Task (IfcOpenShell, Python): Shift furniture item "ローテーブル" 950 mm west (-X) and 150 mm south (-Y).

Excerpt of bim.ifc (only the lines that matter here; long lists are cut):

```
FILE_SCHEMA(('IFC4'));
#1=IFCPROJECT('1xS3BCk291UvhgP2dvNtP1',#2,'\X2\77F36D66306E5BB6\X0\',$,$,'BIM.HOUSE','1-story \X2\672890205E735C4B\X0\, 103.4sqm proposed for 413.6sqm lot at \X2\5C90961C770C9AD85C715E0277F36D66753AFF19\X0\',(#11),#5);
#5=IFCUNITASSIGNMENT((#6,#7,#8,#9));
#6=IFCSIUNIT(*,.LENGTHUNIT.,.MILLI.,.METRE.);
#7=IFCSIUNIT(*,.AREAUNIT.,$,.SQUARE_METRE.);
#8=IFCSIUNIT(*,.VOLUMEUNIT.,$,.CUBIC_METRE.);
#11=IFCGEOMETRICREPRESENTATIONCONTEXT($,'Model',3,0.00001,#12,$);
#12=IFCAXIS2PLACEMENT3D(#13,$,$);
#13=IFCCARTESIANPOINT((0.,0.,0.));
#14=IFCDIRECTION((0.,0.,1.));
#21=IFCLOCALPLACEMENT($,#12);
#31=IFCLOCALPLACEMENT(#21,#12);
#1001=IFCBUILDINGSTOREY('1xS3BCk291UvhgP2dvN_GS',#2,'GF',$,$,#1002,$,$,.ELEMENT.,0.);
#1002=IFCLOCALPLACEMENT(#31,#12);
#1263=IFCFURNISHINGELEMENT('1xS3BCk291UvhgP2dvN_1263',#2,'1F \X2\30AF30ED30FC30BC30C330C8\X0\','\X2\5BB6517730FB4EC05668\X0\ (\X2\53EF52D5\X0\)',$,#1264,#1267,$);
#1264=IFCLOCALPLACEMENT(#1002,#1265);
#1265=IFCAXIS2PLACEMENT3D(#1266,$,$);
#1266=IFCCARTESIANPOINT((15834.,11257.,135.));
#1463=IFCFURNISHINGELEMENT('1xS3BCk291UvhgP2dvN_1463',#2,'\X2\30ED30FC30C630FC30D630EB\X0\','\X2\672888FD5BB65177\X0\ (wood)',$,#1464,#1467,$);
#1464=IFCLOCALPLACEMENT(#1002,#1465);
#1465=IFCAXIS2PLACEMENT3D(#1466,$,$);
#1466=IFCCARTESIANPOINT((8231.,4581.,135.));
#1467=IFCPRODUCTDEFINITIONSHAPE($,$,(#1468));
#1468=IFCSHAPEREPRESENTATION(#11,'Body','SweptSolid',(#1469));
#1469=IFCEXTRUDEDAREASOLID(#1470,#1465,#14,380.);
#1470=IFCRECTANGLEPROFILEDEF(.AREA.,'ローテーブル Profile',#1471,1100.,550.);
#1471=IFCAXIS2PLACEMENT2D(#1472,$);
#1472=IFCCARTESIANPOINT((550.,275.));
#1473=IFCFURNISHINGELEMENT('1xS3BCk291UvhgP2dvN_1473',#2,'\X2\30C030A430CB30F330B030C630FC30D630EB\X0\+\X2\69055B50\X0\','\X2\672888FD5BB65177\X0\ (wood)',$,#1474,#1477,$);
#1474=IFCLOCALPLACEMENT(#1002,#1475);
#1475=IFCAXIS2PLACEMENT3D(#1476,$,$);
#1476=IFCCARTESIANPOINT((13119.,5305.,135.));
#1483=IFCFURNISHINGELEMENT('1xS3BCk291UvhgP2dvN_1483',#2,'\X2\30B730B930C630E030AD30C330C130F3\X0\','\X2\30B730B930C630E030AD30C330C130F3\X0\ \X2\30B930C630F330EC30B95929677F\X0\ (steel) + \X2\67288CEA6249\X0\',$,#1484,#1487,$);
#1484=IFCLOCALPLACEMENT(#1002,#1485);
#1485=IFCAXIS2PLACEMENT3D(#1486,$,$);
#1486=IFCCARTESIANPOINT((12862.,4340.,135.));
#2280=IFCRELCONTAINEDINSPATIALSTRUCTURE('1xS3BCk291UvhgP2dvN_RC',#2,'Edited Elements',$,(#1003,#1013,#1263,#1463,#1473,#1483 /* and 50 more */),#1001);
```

```python
import ifcopenshell
import ifcopenshell.api.geometry
import ifcopenshell.util.placement

model = ifcopenshell.open("bim.ifc")

item = model.by_id(1463)
matrix = ifcopenshell.util.placement.get_local_placement(item.ObjectPlacement)
matrix[0, 3] -= 950.0
matrix[1, 3] -= 150.0
ifcopenshell.api.geometry.edit_object_placement(model, product=item, matrix=matrix, is_si=False)

print(ifcopenshell.util.placement.get_local_placement(item.ObjectPlacement).round(3) + 0.0)

model.write("bim_edited.ifc")
```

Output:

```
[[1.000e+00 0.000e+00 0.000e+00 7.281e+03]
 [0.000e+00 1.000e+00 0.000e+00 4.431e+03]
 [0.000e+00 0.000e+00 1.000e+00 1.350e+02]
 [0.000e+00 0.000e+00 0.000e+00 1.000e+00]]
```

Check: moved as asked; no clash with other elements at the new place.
